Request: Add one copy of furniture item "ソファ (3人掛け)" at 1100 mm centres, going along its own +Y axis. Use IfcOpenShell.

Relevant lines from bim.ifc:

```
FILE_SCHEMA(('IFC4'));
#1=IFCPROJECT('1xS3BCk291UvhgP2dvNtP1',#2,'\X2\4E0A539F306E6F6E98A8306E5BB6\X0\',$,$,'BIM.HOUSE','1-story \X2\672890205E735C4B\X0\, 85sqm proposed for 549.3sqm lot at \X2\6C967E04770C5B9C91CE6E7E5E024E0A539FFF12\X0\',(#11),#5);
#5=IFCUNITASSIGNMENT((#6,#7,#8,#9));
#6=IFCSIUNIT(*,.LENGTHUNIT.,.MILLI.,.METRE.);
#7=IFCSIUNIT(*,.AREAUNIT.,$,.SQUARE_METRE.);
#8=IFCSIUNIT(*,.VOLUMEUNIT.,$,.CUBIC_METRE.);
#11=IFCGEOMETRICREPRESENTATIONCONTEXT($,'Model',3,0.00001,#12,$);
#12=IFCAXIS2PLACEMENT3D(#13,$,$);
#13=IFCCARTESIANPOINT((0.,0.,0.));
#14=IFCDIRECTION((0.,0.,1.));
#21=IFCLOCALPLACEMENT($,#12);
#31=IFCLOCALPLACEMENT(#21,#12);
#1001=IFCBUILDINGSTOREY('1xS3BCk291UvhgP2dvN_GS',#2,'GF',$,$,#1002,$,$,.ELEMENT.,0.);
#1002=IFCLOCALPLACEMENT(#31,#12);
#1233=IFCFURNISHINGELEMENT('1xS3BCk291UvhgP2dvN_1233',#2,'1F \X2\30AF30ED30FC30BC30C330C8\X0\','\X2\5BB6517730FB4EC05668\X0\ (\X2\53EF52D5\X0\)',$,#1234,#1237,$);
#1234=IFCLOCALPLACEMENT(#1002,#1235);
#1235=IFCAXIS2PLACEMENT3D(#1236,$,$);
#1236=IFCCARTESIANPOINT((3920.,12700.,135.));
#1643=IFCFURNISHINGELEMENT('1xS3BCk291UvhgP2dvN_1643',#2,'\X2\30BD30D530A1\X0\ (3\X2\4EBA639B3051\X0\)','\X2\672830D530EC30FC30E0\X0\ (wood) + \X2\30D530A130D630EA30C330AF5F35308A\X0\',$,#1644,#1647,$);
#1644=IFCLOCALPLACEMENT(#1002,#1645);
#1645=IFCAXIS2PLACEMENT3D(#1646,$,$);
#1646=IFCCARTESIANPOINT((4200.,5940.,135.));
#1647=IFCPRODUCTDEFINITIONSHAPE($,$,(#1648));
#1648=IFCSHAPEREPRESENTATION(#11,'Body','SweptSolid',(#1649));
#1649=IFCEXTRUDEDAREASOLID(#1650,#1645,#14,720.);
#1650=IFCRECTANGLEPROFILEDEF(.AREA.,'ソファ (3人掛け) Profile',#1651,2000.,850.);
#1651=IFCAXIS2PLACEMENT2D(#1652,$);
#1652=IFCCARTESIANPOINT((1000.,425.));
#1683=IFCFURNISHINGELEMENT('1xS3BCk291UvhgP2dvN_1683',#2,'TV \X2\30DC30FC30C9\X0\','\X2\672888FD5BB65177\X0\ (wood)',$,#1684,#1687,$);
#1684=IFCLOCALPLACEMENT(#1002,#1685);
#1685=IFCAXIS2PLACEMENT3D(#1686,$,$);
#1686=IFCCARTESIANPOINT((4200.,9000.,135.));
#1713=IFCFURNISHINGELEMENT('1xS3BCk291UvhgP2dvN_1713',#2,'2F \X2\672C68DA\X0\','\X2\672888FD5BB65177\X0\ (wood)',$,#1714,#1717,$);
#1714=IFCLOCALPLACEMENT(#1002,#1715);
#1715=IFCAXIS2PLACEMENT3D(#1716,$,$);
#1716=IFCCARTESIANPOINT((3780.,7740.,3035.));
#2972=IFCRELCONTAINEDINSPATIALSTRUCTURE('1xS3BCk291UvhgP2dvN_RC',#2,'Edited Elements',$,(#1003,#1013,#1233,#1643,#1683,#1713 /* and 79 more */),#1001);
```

```python
import ifcopenshell
import ifcopenshell.api.geometry
import ifcopenshell.api.root
import ifcopenshell.util.element
import ifcopenshell.util.placement
import ifcopenshell.util.unit

model = ifcopenshell.open("bim.ifc")
unit_scale = ifcopenshell.util.unit.calculate_unit_scale(model)


def reuse_history(source, copy):
    """copy_class also copies each property set's owner history, people and application; keep the originals."""
    for rel in copy.IsDefinedBy:
        if rel.is_a("IfcRelDefinesByProperties") and (history := rel.RelatingPropertyDefinition.OwnerHistory):
            rel.RelatingPropertyDefinition.OwnerHistory = source.OwnerHistory
            ifcopenshell.util.element.remove_deep2(model, history)


source = model.by_guid("1xS3BCk291UvhgP2dvN_1643")
base = ifcopenshell.util.placement.get_local_placement(source.ObjectPlacement)
step = base[:3, 1] * 1.1 / unit_scale

for i in range(1, 2):
    copy = ifcopenshell.api.root.copy_class(model, product=source)
    copy.Representation = ifcopenshell.util.element.copy_deep(
        model, source.Representation, exclude=["IfcGeometricRepresentationContext", "IfcRepresentationMap"]
    )
    reuse_history(source, copy)
    matrix = base.copy()
    matrix[:3, 3] += i * step
    print("added at", matrix[:3, 3].round(3) + 0.0)
    ifcopenshell.api.geometry.edit_object_placement(model, product=copy, matrix=matrix, is_si=False)

model.write("bim-out.ifc")
```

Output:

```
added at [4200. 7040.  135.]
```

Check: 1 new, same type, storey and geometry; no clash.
